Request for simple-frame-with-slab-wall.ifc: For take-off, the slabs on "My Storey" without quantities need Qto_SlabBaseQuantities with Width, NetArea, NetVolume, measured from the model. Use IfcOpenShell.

First a look at what the model holds.

```python
import ifcopenshell
import ifcopenshell.util.element
import ifcopenshell.util.unit

model = ifcopenshell.open("simple-frame-with-slab-wall.ifc")
print(model.schema)
for unit_type in ("LENGTHUNIT", "AREAUNIT", "VOLUMEUNIT"):
    print(unit_type, ifcopenshell.util.unit.calculate_unit_scale(model, unit_type))
storey = next(s for s in model.by_type("IfcBuildingStorey") if s.Name == "My Storey")
slabs = [e for e in ifcopenshell.util.element.get_decomposition(storey) if e.is_a("IfcSlab")]
for e in sorted(slabs, key=lambda e: e.id()):
    print(e.id(), e.is_a(), e.Name, list(ifcopenshell.util.element.get_psets(e, qtos_only=True)), sep=" | ")
```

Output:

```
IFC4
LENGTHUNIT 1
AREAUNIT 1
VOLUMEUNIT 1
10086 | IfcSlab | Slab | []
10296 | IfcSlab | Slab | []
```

```python
import ifcopenshell
import ifcopenshell.api.pset
import ifcopenshell.geom
import ifcopenshell.util.element
import ifcopenshell.util.shape
import ifcopenshell.util.unit

model = ifcopenshell.open("simple-frame-with-slab-wall.ifc")
unit_scale = ifcopenshell.util.unit.calculate_unit_scale(model)
area_scale = ifcopenshell.util.unit.calculate_unit_scale(model, "AREAUNIT")
volume_scale = ifcopenshell.util.unit.calculate_unit_scale(model, "VOLUMEUNIT")
settings = ifcopenshell.geom.settings()

storey = next(s for s in model.by_type("IfcBuildingStorey") if s.Name == "My Storey")
slabs = [e for e in ifcopenshell.util.element.get_decomposition(storey) if e.is_a("IfcSlab")]

for e in sorted(slabs, key=lambda e: e.id()):
    if ifcopenshell.util.element.get_psets(e, qtos_only=True, should_inherit=False):
        continue
    # Geometry comes back in metres, in the element's own axes.
    shape = ifcopenshell.geom.create_shape(settings, e)
    values = {
        "Width": ifcopenshell.util.shape.get_z(shape.geometry) / unit_scale,
        "NetArea": ifcopenshell.util.shape.get_footprint_area(shape.geometry) / area_scale,
        "NetVolume": ifcopenshell.util.shape.get_volume(shape.geometry) / volume_scale,
    }
    qto = ifcopenshell.api.pset.add_qto(model, product=e, name="Qto_SlabBaseQuantities")
    ifcopenshell.api.pset.edit_qto(model, qto=qto, properties=values)
    print(e.id(), {k: round(v, 3) for k, v in values.items()})

model.write("simple-frame-with-slab-wall_v2.ifc")
```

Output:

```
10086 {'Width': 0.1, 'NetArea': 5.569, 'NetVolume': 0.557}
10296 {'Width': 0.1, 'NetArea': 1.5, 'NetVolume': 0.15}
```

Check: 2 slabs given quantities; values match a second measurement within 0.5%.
